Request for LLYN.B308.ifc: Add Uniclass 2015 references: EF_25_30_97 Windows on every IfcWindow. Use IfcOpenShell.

First a look at what the model holds.

```python
import ifcopenshell

model = ifcopenshell.open("LLYN.B308.ifc")
print(model.schema)
print("classifications:", [c.Name for c in model.by_type("IfcClassification")])
for ifc_class in ("IfcDoor", "IfcRoof", "IfcStair", "IfcWall", "IfcWindow"):
    print(ifc_class, len(model.by_type(ifc_class)))
```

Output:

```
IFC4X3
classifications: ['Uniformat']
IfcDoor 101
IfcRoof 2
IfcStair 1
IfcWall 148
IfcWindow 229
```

```python
import ifcopenshell
import ifcopenshell.api.classification

model = ifcopenshell.open("LLYN.B308.ifc")

system = ifcopenshell.api.classification.add_classification(model, classification="Uniclass 2015")

codes = {
    "IfcWindow": ("EF_25_30_97", "Windows"),
}
for ifc_class, (code, name) in codes.items():
    products = model.by_type(ifc_class)
    ifcopenshell.api.classification.add_reference(
        model, products=products, classification=system, identification=code, name=name
    )
    print(code, len(products))

model.write("LLYN.B308-out.ifc")
```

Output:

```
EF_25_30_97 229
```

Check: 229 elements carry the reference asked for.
